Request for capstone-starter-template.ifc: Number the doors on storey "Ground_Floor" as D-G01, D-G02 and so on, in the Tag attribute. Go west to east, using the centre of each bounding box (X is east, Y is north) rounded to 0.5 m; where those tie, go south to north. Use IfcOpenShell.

First a look at what the model holds.

```python
import ifcopenshell
import ifcopenshell.util.element
import ifcopenshell.util.placement

model = ifcopenshell.open("capstone-starter-template.ifc")
print(model.schema)
storey = next(s for s in model.by_type("IfcBuildingStorey") if s.Name == "Ground_Floor")
doors = [e for e in ifcopenshell.util.element.get_decomposition(storey) if e.is_a("IfcDoor")]
for e in sorted(doors, key=lambda e: e.id()):
    origin = ifcopenshell.util.placement.get_local_placement(e.ObjectPlacement)[:3, 3]
    print(e.id(), e.Tag, e.Name, origin.round(2) + 0.0, sep=" | ")
```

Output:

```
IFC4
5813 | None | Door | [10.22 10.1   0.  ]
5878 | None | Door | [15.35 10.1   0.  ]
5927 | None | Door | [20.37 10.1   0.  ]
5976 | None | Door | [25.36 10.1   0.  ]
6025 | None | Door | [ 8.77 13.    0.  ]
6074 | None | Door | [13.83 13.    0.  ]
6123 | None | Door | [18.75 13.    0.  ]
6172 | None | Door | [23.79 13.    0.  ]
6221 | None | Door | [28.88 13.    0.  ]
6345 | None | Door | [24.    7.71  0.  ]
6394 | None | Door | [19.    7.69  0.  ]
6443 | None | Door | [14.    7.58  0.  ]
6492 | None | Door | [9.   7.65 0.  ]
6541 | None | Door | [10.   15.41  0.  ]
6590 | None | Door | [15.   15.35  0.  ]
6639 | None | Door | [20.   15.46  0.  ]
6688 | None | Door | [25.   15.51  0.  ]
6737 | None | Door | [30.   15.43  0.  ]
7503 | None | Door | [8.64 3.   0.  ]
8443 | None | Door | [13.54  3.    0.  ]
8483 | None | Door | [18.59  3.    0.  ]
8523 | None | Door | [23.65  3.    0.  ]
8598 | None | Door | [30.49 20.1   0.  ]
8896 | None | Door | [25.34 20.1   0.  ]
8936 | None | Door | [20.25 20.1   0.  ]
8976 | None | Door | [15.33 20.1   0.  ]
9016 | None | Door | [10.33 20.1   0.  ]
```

```python
import ifcopenshell
import ifcopenshell.geom
import ifcopenshell.util.element
import ifcopenshell.util.shape

model = ifcopenshell.open("capstone-starter-template.ifc")
settings = ifcopenshell.geom.settings()
settings.set("use-world-coords", True)


def centre(element):
    shape = ifcopenshell.geom.create_shape(settings, element)
    return ifcopenshell.util.shape.get_bbox_centroid(shape.geometry)


storey = next(s for s in model.by_type("IfcBuildingStorey") if s.Name == "Ground_Floor")
doors = [e for e in ifcopenshell.util.element.get_decomposition(storey) if e.is_a("IfcDoor")]

# Insertion points can sit at a corner or the storey origin, so sort by the geometry (in metres).
centres = {e: centre(e) for e in doors}
doors.sort(key=lambda e: (round(centres[e][0] / 0.5), centres[e][1]))

for i, e in enumerate(doors, start=1):
    number = f"D-G{i:02d}"
    e.Tag = number
    print(e.id(), number)

model.write("capstone-starter-template_rev.ifc")
```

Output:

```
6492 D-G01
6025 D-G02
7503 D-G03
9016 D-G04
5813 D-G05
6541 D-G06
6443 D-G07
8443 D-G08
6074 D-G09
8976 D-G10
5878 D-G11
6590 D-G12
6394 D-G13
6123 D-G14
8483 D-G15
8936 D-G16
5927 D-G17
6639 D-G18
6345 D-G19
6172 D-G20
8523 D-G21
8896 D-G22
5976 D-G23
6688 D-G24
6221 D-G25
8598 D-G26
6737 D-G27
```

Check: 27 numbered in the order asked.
